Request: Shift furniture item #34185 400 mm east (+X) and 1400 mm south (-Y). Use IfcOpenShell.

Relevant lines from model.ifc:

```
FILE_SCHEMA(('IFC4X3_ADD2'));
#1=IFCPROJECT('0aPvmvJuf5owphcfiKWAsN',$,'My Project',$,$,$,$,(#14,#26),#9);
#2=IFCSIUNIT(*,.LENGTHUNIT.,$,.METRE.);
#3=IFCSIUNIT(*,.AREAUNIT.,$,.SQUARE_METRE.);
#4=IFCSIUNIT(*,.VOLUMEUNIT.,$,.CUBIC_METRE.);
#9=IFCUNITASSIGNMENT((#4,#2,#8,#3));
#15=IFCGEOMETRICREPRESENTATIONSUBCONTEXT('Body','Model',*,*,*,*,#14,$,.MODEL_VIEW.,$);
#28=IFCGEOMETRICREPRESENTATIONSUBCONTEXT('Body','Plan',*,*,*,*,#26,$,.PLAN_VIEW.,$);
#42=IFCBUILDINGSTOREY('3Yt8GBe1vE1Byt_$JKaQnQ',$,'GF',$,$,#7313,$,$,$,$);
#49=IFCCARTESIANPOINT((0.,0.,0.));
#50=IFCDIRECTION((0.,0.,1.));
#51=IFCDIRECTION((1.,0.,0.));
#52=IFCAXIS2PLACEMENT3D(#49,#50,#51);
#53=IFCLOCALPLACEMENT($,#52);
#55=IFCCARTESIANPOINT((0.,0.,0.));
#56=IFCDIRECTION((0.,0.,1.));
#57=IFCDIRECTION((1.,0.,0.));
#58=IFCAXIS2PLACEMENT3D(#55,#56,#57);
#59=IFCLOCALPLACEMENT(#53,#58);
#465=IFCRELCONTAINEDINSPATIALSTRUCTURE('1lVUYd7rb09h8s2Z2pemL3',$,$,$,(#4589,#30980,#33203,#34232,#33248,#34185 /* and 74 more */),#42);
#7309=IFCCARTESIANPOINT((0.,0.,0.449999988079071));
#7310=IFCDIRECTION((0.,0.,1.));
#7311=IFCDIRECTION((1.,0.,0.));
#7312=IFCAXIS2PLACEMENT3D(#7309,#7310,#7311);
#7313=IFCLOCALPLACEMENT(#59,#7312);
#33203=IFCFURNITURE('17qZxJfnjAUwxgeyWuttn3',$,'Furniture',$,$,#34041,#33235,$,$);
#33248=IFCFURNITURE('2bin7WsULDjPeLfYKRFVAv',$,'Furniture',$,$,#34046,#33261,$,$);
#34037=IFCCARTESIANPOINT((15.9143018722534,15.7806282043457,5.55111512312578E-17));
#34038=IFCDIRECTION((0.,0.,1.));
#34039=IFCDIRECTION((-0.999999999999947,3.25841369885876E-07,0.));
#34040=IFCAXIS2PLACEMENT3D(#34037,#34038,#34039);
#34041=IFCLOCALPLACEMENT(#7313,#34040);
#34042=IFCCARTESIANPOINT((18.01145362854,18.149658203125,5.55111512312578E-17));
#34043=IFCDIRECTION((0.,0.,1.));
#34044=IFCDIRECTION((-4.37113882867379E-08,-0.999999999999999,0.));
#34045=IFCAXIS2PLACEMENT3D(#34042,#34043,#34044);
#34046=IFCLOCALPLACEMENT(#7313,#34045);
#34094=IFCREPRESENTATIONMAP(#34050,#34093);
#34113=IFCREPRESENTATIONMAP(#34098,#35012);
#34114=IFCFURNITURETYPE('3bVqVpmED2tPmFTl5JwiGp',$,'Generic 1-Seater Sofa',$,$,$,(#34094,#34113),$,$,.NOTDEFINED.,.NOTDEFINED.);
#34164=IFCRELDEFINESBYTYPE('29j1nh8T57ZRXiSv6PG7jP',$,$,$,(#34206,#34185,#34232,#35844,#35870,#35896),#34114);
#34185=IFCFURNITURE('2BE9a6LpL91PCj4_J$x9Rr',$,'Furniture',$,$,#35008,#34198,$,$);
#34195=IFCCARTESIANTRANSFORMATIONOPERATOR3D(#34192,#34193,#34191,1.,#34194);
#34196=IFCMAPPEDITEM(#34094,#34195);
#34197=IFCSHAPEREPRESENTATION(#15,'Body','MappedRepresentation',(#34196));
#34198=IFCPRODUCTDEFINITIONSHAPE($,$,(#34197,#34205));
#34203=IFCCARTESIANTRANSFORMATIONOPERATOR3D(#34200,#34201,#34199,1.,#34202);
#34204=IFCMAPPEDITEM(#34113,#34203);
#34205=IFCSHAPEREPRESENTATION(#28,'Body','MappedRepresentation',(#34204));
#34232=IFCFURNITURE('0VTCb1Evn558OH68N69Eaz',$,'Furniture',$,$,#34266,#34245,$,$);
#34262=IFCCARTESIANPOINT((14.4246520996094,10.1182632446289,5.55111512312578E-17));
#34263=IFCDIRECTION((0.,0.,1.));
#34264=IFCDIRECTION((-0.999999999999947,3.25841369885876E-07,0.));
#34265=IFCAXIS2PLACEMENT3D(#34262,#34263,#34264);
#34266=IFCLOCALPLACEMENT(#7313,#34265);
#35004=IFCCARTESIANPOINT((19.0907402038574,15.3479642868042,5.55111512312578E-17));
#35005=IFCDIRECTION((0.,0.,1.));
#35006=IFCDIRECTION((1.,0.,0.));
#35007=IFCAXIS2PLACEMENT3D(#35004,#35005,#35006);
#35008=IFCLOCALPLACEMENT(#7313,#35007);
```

```python
import ifcopenshell
import ifcopenshell.api.geometry
import ifcopenshell.util.placement
import ifcopenshell.util.unit

model = ifcopenshell.open("model.ifc")
unit_scale = ifcopenshell.util.unit.calculate_unit_scale(model)

item = model.by_guid("2BE9a6LpL91PCj4_J$x9Rr")
matrix = ifcopenshell.util.placement.get_local_placement(item.ObjectPlacement)
matrix[0, 3] += 0.4 / unit_scale
matrix[1, 3] -= 1.4 / unit_scale
ifcopenshell.api.geometry.edit_object_placement(model, product=item, matrix=matrix, is_si=False)

print(ifcopenshell.util.placement.get_local_placement(item.ObjectPlacement).round(3) + 0.0)

model.write("model_rev.ifc")
```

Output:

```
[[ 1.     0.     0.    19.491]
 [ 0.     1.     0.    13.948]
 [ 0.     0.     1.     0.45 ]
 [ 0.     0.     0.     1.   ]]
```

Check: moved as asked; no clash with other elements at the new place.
